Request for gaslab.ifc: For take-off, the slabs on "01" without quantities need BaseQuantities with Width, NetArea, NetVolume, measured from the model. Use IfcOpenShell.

First a look at what the model holds.

```python
import ifcopenshell
import ifcopenshell.util.element
import ifcopenshell.util.unit

model = ifcopenshell.open("gaslab.ifc")
print(model.schema)
for unit_type in ("LENGTHUNIT", "AREAUNIT", "VOLUMEUNIT"):
    print(unit_type, ifcopenshell.util.unit.calculate_unit_scale(model, unit_type))
storey = next(s for s in model.by_type("IfcBuildingStorey") if s.Name == "01")
slabs = [e for e in ifcopenshell.util.element.get_decomposition(storey) if e.is_a("IfcSlab")]
for e in sorted(slabs, key=lambda e: e.id()):
    print(e.id(), e.is_a(), e.Name, list(ifcopenshell.util.element.get_psets(e, qtos_only=True)), sep=" | ")
```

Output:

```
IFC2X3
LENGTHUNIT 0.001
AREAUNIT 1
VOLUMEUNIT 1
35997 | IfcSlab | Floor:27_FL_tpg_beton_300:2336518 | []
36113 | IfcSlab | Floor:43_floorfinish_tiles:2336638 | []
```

```python
import ifcopenshell
import ifcopenshell.api.pset
import ifcopenshell.geom
import ifcopenshell.util.element
import ifcopenshell.util.shape
import ifcopenshell.util.unit

model = ifcopenshell.open("gaslab.ifc")
unit_scale = ifcopenshell.util.unit.calculate_unit_scale(model)
area_scale = ifcopenshell.util.unit.calculate_unit_scale(model, "AREAUNIT")
volume_scale = ifcopenshell.util.unit.calculate_unit_scale(model, "VOLUMEUNIT")
settings = ifcopenshell.geom.settings()

storey = next(s for s in model.by_type("IfcBuildingStorey") if s.Name == "01")
slabs = [e for e in ifcopenshell.util.element.get_decomposition(storey) if e.is_a("IfcSlab")]

for e in sorted(slabs, key=lambda e: e.id()):
    if ifcopenshell.util.element.get_psets(e, qtos_only=True, should_inherit=False):
        continue
    # Geometry comes back in metres, in the element's own axes.
    shape = ifcopenshell.geom.create_shape(settings, e)
    values = {
        "Width": ifcopenshell.util.shape.get_z(shape.geometry) / unit_scale,
        "NetArea": ifcopenshell.util.shape.get_footprint_area(shape.geometry) / area_scale,
        "NetVolume": ifcopenshell.util.shape.get_volume(shape.geometry) / volume_scale,
    }
    qto = ifcopenshell.api.pset.add_qto(model, product=e, name="BaseQuantities")
    ifcopenshell.api.pset.edit_qto(model, qto=qto, properties=values)
    print(e.id(), {k: round(v, 3) for k, v in values.items()})

model.write("gaslab_updated.ifc")
```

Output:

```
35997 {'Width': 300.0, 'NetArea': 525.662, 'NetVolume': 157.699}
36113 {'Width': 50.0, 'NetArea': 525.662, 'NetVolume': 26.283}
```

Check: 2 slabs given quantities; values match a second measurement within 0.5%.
